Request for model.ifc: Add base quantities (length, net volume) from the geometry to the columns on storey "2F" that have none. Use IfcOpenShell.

First a look at what the model holds.

```python
import ifcopenshell
import ifcopenshell.util.element
import ifcopenshell.util.unit

model = ifcopenshell.open("model.ifc")
print(model.schema)
for unit_type in ("LENGTHUNIT", "AREAUNIT", "VOLUMEUNIT"):
    print(unit_type, ifcopenshell.util.unit.calculate_unit_scale(model, unit_type))
storey = next(s for s in model.by_type("IfcBuildingStorey") if s.Name == "2F")
columns = [e for e in ifcopenshell.util.element.get_decomposition(storey) if e.is_a("IfcColumn")]
for e in sorted(columns, key=lambda e: e.id()):
    print(e.id(), e.is_a(), e.Name, list(ifcopenshell.util.element.get_psets(e, qtos_only=True)), sep=" | ")
```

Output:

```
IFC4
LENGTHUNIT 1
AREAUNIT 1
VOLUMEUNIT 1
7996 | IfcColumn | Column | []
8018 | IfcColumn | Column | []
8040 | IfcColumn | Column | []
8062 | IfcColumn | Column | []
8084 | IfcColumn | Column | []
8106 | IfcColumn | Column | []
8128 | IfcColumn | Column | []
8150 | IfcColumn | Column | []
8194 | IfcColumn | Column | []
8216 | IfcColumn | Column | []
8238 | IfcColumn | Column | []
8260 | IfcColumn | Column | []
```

```python
import ifcopenshell
import ifcopenshell.api.pset
import ifcopenshell.geom
import ifcopenshell.util.element
import ifcopenshell.util.shape
import ifcopenshell.util.unit

model = ifcopenshell.open("model.ifc")
unit_scale = ifcopenshell.util.unit.calculate_unit_scale(model)
volume_scale = ifcopenshell.util.unit.calculate_unit_scale(model, "VOLUMEUNIT")
settings = ifcopenshell.geom.settings()

storey = next(s for s in model.by_type("IfcBuildingStorey") if s.Name == "2F")
columns = [e for e in ifcopenshell.util.element.get_decomposition(storey) if e.is_a("IfcColumn")]

for e in sorted(columns, key=lambda e: e.id()):
    if ifcopenshell.util.element.get_psets(e, qtos_only=True, should_inherit=False):
        continue
    # Geometry comes back in metres, in the element's own axes.
    shape = ifcopenshell.geom.create_shape(settings, e)
    values = {
        "Length": ifcopenshell.util.shape.get_z(shape.geometry) / unit_scale,
        "NetVolume": ifcopenshell.util.shape.get_volume(shape.geometry) / volume_scale,
    }
    qto = ifcopenshell.api.pset.add_qto(model, product=e, name="Qto_ColumnBaseQuantities")
    ifcopenshell.api.pset.edit_qto(model, qto=qto, properties=values)
    print(e.id(), {k: round(v, 3) for k, v in values.items()})

model.write("model_v2.ifc")
```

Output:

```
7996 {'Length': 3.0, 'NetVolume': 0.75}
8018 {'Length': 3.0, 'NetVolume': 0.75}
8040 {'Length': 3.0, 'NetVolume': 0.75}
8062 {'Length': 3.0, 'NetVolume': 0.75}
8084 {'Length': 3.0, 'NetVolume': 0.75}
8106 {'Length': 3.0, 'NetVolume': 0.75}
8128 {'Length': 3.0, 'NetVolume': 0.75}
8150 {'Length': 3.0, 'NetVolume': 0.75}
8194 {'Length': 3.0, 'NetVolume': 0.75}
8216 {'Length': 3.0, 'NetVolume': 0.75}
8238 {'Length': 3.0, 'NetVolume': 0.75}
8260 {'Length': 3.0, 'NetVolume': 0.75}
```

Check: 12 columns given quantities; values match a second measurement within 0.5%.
